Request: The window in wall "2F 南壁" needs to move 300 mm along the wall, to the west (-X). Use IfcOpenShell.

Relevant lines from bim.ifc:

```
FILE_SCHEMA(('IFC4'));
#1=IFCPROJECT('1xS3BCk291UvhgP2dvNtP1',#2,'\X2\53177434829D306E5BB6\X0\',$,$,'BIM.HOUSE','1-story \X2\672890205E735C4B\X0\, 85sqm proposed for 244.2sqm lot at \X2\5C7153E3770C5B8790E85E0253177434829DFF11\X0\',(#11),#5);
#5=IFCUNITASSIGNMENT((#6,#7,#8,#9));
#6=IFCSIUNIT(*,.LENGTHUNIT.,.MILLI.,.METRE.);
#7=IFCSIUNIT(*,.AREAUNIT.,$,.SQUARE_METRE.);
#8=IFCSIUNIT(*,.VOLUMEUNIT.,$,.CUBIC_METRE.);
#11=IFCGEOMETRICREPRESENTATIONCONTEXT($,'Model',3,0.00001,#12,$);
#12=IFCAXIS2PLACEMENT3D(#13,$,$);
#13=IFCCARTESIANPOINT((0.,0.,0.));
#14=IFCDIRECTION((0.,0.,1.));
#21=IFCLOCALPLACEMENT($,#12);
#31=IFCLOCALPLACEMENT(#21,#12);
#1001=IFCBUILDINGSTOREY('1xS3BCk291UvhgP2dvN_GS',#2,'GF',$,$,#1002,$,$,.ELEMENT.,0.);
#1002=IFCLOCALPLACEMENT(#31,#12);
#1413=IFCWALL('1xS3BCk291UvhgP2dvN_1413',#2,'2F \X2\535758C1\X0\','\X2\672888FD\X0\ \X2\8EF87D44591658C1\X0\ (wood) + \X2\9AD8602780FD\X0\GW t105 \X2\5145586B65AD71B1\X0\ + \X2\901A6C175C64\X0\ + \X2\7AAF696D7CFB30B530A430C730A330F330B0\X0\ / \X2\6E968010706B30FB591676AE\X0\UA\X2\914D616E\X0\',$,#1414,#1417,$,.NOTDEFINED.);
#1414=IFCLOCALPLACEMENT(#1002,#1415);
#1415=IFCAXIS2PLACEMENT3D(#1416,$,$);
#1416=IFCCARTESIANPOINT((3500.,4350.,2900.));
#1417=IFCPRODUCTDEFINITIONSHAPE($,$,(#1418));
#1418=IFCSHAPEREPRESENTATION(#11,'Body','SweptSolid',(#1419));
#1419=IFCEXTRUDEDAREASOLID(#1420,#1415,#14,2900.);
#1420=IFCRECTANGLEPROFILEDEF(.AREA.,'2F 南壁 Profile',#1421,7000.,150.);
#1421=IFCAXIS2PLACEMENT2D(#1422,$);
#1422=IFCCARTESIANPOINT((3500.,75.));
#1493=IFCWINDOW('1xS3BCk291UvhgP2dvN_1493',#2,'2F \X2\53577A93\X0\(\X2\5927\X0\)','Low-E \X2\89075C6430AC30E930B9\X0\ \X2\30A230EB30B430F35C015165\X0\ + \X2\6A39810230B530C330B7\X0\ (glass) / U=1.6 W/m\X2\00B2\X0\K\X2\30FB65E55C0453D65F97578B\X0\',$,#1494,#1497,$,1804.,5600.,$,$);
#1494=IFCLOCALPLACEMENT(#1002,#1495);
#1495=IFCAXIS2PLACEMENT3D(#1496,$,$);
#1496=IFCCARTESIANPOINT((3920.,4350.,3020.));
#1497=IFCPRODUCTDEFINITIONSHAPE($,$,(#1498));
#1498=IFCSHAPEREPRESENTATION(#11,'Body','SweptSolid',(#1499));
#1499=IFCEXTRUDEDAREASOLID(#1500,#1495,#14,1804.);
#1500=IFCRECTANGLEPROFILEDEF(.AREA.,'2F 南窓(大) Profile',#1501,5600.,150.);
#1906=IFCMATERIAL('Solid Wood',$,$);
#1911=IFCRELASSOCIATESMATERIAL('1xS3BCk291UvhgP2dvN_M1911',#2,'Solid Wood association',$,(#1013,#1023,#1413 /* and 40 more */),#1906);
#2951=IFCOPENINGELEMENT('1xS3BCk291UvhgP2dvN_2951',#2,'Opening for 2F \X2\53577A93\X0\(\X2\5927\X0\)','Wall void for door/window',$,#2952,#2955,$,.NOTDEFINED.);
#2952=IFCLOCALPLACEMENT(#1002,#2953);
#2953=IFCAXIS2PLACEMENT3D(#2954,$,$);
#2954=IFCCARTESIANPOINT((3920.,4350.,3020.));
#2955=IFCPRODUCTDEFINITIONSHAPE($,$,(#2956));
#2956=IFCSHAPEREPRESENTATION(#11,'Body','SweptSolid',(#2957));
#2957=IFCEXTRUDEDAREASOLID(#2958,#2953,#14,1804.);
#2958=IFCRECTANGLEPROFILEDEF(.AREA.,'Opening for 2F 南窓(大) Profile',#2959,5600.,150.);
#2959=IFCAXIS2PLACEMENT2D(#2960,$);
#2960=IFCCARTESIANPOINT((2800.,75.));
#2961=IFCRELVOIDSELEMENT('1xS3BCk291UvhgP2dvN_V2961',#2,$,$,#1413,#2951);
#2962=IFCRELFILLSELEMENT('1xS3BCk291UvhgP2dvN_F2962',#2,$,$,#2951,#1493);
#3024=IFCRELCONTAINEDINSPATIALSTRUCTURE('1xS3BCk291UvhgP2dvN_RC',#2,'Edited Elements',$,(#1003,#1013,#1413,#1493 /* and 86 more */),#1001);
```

```python
import ifcopenshell
import ifcopenshell.api.geometry
import ifcopenshell.util.placement

model = ifcopenshell.open("bim.ifc")

window = model.by_id(1493)
opening = window.FillsVoids[0].RelatingOpeningElement
wall = opening.VoidsElements[0].RelatingBuildingElement

wall_matrix = ifcopenshell.util.placement.get_local_placement(wall.ObjectPlacement)
shift = wall_matrix[:3, 0] * -300.0
before = ifcopenshell.util.placement.get_local_placement(window.ObjectPlacement)[:3, 3].copy()

# The window is not placed relative to its opening, so move both.
for product in (opening, window):
    matrix = ifcopenshell.util.placement.get_local_placement(product.ObjectPlacement)
    matrix[:3, 3] += shift
    ifcopenshell.api.geometry.edit_object_placement(model, product=product, matrix=matrix, is_si=False)

after = ifcopenshell.util.placement.get_local_placement(window.ObjectPlacement)[:3, 3]
print("window moved by", (after - before).round(3) + 0.0)

model.write("bim_v2.ifc")
```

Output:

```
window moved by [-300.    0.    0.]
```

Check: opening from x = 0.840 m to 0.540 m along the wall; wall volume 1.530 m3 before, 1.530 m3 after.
